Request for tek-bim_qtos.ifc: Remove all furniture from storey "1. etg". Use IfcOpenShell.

First a look at what the model holds.

```python
import ifcopenshell
import ifcopenshell.util.element

model = ifcopenshell.open("tek-bim_qtos.ifc")
print(model.schema)
storey = next(s for s in model.by_type("IfcBuildingStorey") if s.Name == "1. etg")
furniture = [e for e in ifcopenshell.util.element.get_decomposition(storey) if e.is_a("IfcFurnishingElement")]
seen = {}
for e in furniture:
    element_type = ifcopenshell.util.element.get_type(e)
    name = element_type.Name if element_type not in (None, e) else None
    seen[name] = seen.get(name, 0) + 1
for name, count in sorted(seen.items(), key=str):
    print(count, "x", name)
```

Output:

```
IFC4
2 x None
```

```python
import ifcopenshell
import ifcopenshell.api.root
import ifcopenshell.util.element

model = ifcopenshell.open("tek-bim_qtos.ifc")

storey = next(s for s in model.by_type("IfcBuildingStorey") if s.Name == "1. etg")
furniture = [e for e in ifcopenshell.util.element.get_decomposition(storey) if e.is_a("IfcFurnishingElement")]

for e in furniture:
    ifcopenshell.api.root.remove_product(model, product=e)
print(len(furniture), "removed")

model.write("tek-bim_qtos_updated.ifc")
```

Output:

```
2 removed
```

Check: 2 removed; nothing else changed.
